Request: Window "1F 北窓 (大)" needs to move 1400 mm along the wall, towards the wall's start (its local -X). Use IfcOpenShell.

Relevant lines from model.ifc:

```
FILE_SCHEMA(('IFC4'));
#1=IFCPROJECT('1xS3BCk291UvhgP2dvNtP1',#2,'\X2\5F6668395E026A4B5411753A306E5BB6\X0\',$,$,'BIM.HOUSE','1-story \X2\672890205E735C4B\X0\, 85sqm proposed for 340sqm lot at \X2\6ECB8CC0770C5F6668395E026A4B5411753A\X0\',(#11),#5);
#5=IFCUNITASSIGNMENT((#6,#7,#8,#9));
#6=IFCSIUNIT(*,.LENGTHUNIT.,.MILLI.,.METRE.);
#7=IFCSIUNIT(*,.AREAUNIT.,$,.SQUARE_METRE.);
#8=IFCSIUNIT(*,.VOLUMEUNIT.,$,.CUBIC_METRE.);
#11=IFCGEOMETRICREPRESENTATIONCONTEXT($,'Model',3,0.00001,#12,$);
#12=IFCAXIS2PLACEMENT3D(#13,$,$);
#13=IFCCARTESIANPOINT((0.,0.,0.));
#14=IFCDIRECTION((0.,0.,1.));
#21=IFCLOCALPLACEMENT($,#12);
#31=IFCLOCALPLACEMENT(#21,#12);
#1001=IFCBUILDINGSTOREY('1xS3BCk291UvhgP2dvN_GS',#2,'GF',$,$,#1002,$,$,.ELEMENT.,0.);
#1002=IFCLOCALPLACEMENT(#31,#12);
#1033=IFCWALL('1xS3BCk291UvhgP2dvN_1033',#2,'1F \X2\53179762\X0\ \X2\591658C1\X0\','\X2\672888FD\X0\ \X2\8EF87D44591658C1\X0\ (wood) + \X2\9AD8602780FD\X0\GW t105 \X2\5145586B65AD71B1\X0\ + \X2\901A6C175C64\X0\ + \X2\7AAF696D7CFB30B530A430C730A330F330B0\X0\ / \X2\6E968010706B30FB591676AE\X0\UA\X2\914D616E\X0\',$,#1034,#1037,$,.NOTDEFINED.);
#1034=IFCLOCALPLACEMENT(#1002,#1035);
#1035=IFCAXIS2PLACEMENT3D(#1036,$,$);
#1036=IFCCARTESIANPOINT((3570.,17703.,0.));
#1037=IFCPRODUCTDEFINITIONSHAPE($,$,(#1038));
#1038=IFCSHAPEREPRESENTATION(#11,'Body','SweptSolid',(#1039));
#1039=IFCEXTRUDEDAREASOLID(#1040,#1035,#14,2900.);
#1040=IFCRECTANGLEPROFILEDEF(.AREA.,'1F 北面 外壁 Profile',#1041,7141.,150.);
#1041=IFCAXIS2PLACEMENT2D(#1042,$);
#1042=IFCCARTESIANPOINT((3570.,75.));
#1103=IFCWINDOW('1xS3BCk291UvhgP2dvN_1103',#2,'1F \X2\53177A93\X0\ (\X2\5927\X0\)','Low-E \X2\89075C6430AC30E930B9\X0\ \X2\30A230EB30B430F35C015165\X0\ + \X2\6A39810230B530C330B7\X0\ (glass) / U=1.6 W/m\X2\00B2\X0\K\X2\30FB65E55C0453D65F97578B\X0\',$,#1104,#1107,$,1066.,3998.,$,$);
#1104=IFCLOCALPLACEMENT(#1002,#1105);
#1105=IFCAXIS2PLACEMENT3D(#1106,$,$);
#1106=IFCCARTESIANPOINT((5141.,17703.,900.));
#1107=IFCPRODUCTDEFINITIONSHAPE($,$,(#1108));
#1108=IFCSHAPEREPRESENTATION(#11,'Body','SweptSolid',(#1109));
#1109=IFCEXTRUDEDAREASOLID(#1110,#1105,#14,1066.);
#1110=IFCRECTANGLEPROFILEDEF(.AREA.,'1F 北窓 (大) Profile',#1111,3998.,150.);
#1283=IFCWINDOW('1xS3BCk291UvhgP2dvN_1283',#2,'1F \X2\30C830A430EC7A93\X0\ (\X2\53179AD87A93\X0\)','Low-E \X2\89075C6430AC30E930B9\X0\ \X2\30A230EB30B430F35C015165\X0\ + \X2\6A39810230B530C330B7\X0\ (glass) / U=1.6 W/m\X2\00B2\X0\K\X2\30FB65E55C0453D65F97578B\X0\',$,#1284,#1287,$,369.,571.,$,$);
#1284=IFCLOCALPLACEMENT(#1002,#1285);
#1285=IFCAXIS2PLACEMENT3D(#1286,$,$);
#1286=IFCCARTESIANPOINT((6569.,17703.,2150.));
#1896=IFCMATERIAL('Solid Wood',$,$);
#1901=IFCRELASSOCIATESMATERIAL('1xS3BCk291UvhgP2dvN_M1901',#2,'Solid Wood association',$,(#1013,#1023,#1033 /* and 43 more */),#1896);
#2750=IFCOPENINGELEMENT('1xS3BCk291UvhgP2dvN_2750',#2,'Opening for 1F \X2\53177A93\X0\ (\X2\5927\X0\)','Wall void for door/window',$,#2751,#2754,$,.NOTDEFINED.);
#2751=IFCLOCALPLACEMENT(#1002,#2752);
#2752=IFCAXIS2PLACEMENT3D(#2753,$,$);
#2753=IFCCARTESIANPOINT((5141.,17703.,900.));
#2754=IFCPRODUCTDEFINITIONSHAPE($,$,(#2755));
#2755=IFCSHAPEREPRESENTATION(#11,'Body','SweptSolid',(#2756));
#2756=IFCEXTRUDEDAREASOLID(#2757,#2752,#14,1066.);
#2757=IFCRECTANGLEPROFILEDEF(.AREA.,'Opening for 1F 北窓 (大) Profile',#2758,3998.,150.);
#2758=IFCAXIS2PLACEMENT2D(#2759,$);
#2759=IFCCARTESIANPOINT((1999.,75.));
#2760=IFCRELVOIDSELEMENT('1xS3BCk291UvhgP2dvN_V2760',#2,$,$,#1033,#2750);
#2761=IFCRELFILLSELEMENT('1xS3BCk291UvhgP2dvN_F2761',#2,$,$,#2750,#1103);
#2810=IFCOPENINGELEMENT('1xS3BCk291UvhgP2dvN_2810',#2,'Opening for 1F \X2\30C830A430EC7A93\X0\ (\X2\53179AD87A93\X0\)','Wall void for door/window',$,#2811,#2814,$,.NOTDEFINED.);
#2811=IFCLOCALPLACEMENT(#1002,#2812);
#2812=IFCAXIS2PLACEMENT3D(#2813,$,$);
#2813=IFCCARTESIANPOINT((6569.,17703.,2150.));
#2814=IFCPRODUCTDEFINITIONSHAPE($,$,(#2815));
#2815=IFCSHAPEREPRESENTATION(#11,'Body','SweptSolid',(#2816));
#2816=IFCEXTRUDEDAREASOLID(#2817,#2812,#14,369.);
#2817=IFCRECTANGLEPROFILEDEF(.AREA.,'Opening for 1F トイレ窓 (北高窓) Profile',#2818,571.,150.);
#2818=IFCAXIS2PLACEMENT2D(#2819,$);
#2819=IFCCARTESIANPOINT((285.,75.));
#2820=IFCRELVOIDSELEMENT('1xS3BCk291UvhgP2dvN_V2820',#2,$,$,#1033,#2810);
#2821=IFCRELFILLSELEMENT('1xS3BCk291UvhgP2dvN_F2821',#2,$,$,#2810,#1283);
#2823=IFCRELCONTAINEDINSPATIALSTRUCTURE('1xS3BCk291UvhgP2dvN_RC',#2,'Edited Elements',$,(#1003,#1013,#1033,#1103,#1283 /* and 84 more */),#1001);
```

```python
import ifcopenshell
import ifcopenshell.api.geometry
import ifcopenshell.util.placement
import ifcopenshell.util.unit

model = ifcopenshell.open("model.ifc")
unit_scale = ifcopenshell.util.unit.calculate_unit_scale(model)

window = model.by_guid("1xS3BCk291UvhgP2dvN_1103")
opening = window.FillsVoids[0].RelatingOpeningElement
wall = opening.VoidsElements[0].RelatingBuildingElement

wall_matrix = ifcopenshell.util.placement.get_local_placement(wall.ObjectPlacement)
shift = wall_matrix[:3, 0] * -1.4 / unit_scale
before = ifcopenshell.util.placement.get_local_placement(window.ObjectPlacement)[:3, 3].copy()

# The window is not placed relative to its opening, so move both.
for product in (opening, window):
    matrix = ifcopenshell.util.placement.get_local_placement(product.ObjectPlacement)
    matrix[:3, 3] += shift
    ifcopenshell.api.geometry.edit_object_placement(model, product=product, matrix=matrix, is_si=False)

after = ifcopenshell.util.placement.get_local_placement(window.ObjectPlacement)[:3, 3]
print("window moved by", (after - before).round(3) + 0.0)

model.write("model_updated.ifc")
```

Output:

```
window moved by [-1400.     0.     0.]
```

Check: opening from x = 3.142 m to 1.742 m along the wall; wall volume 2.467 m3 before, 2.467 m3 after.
